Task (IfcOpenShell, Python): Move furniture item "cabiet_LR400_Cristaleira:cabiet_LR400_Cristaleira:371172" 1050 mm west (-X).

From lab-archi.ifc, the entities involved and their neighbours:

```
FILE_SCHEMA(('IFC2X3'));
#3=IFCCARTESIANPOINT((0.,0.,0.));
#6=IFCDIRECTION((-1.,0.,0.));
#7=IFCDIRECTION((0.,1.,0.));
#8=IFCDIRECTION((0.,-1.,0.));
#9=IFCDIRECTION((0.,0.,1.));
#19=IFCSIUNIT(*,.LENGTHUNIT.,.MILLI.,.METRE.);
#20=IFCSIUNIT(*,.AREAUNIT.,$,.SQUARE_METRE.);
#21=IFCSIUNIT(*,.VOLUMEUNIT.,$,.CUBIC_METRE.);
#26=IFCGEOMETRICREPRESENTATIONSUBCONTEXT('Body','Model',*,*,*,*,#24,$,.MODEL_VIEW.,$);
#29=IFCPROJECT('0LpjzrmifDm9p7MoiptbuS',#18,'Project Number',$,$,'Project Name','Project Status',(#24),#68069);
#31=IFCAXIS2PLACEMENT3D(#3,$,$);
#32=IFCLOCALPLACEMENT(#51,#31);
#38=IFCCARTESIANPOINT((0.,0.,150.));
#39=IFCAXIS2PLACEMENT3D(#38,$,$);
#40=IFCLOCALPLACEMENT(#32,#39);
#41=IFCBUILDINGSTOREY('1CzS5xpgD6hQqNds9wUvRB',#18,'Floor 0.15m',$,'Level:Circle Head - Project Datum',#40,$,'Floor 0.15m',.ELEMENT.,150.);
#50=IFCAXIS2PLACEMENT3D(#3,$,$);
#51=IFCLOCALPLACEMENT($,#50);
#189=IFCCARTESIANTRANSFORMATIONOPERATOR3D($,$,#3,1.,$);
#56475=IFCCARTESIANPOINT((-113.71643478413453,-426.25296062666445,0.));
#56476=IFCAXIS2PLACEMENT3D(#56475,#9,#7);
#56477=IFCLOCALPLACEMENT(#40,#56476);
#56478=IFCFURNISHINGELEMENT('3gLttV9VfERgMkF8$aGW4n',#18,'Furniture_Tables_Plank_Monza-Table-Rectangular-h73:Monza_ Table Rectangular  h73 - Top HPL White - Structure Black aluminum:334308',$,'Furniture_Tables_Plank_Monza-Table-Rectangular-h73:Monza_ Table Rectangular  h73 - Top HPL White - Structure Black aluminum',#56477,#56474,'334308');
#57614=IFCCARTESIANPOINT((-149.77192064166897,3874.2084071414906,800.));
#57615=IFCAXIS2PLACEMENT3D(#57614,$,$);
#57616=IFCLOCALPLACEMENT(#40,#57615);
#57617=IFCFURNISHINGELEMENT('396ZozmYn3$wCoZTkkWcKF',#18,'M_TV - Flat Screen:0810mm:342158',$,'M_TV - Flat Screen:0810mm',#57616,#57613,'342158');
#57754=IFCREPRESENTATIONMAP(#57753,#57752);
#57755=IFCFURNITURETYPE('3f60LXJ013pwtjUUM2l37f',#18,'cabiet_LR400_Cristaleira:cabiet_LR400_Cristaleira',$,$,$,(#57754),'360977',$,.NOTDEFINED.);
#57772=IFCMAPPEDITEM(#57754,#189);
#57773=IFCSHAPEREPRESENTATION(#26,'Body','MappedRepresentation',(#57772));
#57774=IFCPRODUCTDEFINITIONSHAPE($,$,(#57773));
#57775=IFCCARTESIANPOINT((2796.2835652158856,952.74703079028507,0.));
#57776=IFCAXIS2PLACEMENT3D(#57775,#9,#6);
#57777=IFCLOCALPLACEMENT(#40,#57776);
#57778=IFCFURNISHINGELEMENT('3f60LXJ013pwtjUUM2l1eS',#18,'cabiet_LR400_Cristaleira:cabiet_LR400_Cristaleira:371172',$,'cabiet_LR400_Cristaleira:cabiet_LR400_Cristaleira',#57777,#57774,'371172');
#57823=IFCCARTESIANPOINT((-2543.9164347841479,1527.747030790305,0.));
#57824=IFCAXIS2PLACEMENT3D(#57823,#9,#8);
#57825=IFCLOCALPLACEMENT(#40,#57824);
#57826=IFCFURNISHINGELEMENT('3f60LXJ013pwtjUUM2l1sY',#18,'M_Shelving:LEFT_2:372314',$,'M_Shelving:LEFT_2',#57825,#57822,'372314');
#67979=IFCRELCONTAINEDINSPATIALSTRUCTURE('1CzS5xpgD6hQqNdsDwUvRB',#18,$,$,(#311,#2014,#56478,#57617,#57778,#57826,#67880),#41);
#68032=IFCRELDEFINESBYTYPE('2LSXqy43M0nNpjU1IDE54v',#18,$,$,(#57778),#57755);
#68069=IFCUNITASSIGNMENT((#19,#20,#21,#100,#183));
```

```python
import ifcopenshell
import ifcopenshell.api.geometry
import ifcopenshell.util.placement
import ifcopenshell.util.unit

model = ifcopenshell.open("lab-archi.ifc")
unit_scale = ifcopenshell.util.unit.calculate_unit_scale(model)

item = model.by_id(57778)
matrix = ifcopenshell.util.placement.get_local_placement(item.ObjectPlacement)
matrix[0, 3] -= 1.05 / unit_scale
ifcopenshell.api.geometry.edit_object_placement(model, product=item, matrix=matrix, is_si=False)

print(ifcopenshell.util.placement.get_local_placement(item.ObjectPlacement).round(3) + 0.0)

model.write("lab-archi_rev.ifc")
```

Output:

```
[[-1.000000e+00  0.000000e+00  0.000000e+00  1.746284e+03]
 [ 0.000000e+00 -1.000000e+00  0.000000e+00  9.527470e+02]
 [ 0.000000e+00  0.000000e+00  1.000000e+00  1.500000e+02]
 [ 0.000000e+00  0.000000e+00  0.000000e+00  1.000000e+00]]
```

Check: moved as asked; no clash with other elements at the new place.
